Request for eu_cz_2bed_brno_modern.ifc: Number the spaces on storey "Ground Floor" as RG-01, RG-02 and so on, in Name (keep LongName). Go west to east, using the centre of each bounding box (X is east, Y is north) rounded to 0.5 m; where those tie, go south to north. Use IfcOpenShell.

First a look at what the model holds.

```python
import ifcopenshell
import ifcopenshell.util.element
import ifcopenshell.util.placement

model = ifcopenshell.open("eu_cz_2bed_brno_modern.ifc")
print(model.schema)
storey = next(s for s in model.by_type("IfcBuildingStorey") if s.Name == "Ground Floor")
spaces = [e for e in ifcopenshell.util.element.get_decomposition(storey) if e.is_a("IfcSpace")]
for e in sorted(spaces, key=lambda e: e.id()):
    origin = ifcopenshell.util.placement.get_local_placement(e.ObjectPlacement)[:3, 3]
    print(e.id(), e.Name, e.LongName, origin.round(2) + 0.0, sep=" | ")
```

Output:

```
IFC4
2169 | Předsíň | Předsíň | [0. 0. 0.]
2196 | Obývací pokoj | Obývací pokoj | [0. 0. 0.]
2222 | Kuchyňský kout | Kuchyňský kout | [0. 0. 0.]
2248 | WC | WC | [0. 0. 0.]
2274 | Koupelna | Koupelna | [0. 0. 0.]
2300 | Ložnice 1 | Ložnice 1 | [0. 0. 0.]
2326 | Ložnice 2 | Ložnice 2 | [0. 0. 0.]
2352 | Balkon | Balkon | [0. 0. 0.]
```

```python
import ifcopenshell
import ifcopenshell.geom
import ifcopenshell.util.element
import ifcopenshell.util.shape

model = ifcopenshell.open("eu_cz_2bed_brno_modern.ifc")
settings = ifcopenshell.geom.settings()
settings.set("use-world-coords", True)


def centre(element):
    shape = ifcopenshell.geom.create_shape(settings, element)
    return ifcopenshell.util.shape.get_bbox_centroid(shape.geometry)


storey = next(s for s in model.by_type("IfcBuildingStorey") if s.Name == "Ground Floor")
spaces = [e for e in ifcopenshell.util.element.get_decomposition(storey) if e.is_a("IfcSpace")]

# Insertion points can sit at a corner or the storey origin, so sort by the geometry (in metres).
centres = {e: centre(e) for e in spaces}
spaces.sort(key=lambda e: (round(centres[e][0] / 0.5), centres[e][1]))

for i, e in enumerate(spaces, start=1):
    number = f"RG-{i:02d}"
    e.Name = number
    print(e.id(), number)

model.write("eu_cz_2bed_brno_modern_updated.ifc")
```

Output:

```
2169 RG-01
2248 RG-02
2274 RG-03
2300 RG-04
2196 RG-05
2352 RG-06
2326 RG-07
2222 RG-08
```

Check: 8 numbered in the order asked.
